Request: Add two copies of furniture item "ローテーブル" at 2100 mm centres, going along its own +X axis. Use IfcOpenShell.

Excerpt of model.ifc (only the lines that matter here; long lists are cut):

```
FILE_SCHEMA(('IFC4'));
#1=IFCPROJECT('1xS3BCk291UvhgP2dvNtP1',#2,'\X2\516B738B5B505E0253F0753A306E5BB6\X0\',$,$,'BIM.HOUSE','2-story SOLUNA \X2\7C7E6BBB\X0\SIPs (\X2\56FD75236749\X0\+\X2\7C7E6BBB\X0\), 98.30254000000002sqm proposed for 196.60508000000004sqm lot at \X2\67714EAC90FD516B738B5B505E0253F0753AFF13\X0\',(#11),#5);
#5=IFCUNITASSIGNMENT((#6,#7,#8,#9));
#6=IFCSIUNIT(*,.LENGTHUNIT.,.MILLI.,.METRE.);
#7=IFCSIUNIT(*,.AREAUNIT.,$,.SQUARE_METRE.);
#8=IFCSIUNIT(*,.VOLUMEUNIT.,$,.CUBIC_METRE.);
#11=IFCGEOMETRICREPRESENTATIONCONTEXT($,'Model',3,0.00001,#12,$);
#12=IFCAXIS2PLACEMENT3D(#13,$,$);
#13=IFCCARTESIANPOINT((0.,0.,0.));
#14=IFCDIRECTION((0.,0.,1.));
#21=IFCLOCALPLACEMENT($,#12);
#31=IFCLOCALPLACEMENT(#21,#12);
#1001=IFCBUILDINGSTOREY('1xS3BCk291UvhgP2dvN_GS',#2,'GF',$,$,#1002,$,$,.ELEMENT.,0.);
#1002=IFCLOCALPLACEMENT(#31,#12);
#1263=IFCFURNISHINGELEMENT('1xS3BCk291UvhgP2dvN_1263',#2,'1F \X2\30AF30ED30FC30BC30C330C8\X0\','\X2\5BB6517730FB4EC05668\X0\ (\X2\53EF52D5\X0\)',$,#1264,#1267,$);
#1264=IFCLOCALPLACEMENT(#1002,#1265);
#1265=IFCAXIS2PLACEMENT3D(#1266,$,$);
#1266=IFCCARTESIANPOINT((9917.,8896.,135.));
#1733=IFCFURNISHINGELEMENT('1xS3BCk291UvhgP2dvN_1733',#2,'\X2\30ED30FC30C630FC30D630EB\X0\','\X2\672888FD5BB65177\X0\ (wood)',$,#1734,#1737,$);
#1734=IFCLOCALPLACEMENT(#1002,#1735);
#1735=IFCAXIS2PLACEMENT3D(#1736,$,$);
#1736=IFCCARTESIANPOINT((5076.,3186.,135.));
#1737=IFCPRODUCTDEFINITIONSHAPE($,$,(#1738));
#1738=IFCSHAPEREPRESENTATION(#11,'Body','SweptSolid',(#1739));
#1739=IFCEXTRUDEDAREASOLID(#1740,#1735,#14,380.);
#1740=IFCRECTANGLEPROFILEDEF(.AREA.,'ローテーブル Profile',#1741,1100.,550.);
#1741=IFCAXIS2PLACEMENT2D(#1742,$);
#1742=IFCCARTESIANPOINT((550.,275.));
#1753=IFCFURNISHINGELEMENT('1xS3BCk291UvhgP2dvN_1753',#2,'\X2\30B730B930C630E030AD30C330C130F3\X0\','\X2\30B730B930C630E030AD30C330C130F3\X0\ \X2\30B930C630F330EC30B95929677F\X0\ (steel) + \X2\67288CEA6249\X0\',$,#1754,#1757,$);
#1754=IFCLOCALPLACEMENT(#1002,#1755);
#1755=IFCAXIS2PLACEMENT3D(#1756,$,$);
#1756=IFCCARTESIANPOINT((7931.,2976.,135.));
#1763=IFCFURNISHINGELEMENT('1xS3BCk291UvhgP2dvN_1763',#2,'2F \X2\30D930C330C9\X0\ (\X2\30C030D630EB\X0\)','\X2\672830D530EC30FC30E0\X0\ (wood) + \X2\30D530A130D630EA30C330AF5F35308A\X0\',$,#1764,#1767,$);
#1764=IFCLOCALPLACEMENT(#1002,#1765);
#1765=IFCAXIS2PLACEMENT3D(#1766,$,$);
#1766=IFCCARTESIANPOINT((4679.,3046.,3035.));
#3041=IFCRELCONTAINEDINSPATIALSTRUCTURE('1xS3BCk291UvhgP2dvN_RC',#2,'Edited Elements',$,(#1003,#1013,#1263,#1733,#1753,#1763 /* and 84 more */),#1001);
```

```python
import ifcopenshell
import ifcopenshell.api.geometry
import ifcopenshell.api.root
import ifcopenshell.util.element
import ifcopenshell.util.placement
import ifcopenshell.util.unit

model = ifcopenshell.open("model.ifc")
unit_scale = ifcopenshell.util.unit.calculate_unit_scale(model)


def reuse_history(source, copy):
    """copy_class also copies each property set's owner history, people and application; keep the originals."""
    for rel in copy.IsDefinedBy:
        if rel.is_a("IfcRelDefinesByProperties") and (history := rel.RelatingPropertyDefinition.OwnerHistory):
            rel.RelatingPropertyDefinition.OwnerHistory = source.OwnerHistory
            ifcopenshell.util.element.remove_deep2(model, history)


source = model.by_guid("1xS3BCk291UvhgP2dvN_1733")
base = ifcopenshell.util.placement.get_local_placement(source.ObjectPlacement)
step = base[:3, 0] * 2.1 / unit_scale

for i in range(1, 3):
    copy = ifcopenshell.api.root.copy_class(model, product=source)
    copy.Representation = ifcopenshell.util.element.copy_deep(
        model, source.Representation, exclude=["IfcGeometricRepresentationContext", "IfcRepresentationMap"]
    )
    reuse_history(source, copy)
    matrix = base.copy()
    matrix[:3, 3] += i * step
    print("added at", matrix[:3, 3].round(3) + 0.0)
    ifcopenshell.api.geometry.edit_object_placement(model, product=copy, matrix=matrix, is_si=False)

model.write("model_v2.ifc")
```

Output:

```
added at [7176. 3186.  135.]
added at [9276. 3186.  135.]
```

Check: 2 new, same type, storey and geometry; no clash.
